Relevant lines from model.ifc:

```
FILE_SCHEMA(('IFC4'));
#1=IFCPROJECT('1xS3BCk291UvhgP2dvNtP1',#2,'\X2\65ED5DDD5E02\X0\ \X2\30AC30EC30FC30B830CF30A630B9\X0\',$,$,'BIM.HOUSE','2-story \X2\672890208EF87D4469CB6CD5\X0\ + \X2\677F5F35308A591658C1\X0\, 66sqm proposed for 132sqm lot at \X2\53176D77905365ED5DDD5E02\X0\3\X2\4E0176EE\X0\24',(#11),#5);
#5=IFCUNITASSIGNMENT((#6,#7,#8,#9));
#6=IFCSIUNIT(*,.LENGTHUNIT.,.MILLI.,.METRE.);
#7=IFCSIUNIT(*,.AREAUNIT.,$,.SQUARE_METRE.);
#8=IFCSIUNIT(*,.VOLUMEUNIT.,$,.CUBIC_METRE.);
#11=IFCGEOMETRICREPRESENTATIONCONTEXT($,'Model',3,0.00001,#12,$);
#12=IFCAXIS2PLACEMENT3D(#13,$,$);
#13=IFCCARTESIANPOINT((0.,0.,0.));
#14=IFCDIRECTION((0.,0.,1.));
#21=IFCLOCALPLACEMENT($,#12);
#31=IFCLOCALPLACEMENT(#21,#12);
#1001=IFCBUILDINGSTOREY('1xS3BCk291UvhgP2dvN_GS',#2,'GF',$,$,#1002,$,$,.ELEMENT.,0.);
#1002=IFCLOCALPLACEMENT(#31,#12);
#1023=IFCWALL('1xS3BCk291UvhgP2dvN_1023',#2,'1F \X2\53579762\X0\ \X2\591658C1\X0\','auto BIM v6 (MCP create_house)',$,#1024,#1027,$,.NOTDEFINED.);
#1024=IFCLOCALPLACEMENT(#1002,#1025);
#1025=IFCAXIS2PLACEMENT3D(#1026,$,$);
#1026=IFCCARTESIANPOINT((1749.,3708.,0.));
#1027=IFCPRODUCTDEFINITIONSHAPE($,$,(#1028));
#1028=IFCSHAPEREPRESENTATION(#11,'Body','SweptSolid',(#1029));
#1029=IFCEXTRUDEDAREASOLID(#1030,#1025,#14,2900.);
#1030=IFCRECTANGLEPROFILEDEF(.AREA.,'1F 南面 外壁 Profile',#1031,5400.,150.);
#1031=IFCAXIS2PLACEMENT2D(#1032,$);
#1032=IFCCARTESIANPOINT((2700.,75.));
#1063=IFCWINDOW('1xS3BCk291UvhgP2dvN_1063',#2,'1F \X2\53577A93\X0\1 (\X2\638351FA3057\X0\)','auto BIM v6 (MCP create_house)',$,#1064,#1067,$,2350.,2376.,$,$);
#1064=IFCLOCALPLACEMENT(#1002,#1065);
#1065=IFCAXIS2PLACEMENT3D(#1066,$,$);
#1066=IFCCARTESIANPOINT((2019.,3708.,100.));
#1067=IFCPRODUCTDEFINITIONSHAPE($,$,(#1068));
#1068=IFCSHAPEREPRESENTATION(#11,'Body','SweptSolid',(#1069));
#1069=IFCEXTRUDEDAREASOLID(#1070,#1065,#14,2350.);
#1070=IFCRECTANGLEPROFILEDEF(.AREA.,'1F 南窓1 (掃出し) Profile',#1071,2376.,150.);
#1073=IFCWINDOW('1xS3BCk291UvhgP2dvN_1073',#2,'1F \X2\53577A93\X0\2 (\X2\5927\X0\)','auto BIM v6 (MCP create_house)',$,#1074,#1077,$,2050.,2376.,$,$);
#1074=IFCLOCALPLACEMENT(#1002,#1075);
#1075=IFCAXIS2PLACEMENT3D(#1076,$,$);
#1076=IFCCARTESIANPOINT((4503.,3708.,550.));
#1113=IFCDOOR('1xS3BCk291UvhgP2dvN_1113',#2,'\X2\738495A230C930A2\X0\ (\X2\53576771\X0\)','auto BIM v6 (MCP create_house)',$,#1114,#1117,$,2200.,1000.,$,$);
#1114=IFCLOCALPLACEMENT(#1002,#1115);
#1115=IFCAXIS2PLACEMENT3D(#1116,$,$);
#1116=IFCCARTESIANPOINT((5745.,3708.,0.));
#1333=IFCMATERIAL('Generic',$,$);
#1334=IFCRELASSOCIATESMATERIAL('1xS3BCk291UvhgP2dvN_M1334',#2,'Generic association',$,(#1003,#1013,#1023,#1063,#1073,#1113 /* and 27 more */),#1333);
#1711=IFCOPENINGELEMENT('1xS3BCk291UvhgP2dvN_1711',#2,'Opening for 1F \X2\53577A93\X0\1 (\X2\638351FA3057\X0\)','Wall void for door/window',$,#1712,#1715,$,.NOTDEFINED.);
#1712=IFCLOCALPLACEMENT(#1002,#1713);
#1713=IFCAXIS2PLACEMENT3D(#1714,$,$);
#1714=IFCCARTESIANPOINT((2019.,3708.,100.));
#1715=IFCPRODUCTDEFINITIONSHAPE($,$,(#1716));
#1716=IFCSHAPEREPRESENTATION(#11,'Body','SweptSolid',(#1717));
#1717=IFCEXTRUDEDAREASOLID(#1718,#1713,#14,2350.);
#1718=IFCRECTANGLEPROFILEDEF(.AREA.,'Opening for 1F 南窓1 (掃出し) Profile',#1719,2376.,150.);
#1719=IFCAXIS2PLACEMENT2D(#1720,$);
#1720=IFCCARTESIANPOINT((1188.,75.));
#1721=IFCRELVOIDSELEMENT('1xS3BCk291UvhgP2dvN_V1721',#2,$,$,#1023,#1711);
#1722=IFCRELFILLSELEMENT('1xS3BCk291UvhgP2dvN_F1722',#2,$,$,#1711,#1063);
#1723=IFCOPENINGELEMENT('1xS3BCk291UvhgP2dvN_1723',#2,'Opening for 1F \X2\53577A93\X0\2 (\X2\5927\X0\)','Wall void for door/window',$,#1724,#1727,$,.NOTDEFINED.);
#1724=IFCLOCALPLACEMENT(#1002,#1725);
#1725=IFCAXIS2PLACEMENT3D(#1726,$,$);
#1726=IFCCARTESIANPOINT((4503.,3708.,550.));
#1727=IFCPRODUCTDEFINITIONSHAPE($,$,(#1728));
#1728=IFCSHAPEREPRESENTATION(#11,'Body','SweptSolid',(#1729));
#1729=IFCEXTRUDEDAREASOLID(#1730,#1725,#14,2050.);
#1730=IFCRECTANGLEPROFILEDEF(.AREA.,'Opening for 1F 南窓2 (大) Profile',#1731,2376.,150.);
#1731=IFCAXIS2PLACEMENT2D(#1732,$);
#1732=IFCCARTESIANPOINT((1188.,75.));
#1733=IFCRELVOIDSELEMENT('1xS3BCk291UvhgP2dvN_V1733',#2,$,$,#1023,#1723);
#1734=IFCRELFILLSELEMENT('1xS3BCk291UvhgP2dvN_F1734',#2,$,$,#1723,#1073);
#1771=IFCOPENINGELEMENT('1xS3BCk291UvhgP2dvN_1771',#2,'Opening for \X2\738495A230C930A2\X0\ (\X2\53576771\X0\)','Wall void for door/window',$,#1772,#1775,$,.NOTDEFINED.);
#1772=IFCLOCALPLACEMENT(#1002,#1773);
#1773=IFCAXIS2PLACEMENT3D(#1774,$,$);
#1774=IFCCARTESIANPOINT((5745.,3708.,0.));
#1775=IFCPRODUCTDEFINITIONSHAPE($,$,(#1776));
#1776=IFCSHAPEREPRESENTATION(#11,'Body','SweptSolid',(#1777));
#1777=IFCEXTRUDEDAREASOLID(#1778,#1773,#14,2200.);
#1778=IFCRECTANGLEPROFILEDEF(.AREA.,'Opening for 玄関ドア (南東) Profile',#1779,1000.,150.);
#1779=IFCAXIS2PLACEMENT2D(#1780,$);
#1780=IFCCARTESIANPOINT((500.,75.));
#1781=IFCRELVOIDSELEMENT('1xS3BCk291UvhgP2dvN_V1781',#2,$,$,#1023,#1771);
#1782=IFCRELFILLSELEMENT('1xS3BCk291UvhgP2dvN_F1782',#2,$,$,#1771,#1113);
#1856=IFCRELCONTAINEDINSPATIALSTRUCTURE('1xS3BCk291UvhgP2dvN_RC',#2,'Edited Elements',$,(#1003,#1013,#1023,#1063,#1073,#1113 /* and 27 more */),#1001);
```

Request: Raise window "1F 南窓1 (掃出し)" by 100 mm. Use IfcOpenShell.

```python
import numpy as np
import ifcopenshell
import ifcopenshell.api.geometry
import ifcopenshell.util.placement
import ifcopenshell.util.unit

model = ifcopenshell.open("model.ifc")
unit_scale = ifcopenshell.util.unit.calculate_unit_scale(model)

window = model.by_guid("1xS3BCk291UvhgP2dvN_1063")
opening = window.FillsVoids[0].RelatingOpeningElement
dz = 0.1 / unit_scale

shift = np.array([0.0, 0.0, dz])
# The window is not placed relative to its opening, so move both.
for product in (opening, window):
    matrix = ifcopenshell.util.placement.get_local_placement(product.ObjectPlacement)
    matrix[:3, 3] += shift
    ifcopenshell.api.geometry.edit_object_placement(model, product=product, matrix=matrix, is_si=False)

print(f"moved by {dz * unit_scale:+.3f} m")

model.write("model_v2.ifc")
```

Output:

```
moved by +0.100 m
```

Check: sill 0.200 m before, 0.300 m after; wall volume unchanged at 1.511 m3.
